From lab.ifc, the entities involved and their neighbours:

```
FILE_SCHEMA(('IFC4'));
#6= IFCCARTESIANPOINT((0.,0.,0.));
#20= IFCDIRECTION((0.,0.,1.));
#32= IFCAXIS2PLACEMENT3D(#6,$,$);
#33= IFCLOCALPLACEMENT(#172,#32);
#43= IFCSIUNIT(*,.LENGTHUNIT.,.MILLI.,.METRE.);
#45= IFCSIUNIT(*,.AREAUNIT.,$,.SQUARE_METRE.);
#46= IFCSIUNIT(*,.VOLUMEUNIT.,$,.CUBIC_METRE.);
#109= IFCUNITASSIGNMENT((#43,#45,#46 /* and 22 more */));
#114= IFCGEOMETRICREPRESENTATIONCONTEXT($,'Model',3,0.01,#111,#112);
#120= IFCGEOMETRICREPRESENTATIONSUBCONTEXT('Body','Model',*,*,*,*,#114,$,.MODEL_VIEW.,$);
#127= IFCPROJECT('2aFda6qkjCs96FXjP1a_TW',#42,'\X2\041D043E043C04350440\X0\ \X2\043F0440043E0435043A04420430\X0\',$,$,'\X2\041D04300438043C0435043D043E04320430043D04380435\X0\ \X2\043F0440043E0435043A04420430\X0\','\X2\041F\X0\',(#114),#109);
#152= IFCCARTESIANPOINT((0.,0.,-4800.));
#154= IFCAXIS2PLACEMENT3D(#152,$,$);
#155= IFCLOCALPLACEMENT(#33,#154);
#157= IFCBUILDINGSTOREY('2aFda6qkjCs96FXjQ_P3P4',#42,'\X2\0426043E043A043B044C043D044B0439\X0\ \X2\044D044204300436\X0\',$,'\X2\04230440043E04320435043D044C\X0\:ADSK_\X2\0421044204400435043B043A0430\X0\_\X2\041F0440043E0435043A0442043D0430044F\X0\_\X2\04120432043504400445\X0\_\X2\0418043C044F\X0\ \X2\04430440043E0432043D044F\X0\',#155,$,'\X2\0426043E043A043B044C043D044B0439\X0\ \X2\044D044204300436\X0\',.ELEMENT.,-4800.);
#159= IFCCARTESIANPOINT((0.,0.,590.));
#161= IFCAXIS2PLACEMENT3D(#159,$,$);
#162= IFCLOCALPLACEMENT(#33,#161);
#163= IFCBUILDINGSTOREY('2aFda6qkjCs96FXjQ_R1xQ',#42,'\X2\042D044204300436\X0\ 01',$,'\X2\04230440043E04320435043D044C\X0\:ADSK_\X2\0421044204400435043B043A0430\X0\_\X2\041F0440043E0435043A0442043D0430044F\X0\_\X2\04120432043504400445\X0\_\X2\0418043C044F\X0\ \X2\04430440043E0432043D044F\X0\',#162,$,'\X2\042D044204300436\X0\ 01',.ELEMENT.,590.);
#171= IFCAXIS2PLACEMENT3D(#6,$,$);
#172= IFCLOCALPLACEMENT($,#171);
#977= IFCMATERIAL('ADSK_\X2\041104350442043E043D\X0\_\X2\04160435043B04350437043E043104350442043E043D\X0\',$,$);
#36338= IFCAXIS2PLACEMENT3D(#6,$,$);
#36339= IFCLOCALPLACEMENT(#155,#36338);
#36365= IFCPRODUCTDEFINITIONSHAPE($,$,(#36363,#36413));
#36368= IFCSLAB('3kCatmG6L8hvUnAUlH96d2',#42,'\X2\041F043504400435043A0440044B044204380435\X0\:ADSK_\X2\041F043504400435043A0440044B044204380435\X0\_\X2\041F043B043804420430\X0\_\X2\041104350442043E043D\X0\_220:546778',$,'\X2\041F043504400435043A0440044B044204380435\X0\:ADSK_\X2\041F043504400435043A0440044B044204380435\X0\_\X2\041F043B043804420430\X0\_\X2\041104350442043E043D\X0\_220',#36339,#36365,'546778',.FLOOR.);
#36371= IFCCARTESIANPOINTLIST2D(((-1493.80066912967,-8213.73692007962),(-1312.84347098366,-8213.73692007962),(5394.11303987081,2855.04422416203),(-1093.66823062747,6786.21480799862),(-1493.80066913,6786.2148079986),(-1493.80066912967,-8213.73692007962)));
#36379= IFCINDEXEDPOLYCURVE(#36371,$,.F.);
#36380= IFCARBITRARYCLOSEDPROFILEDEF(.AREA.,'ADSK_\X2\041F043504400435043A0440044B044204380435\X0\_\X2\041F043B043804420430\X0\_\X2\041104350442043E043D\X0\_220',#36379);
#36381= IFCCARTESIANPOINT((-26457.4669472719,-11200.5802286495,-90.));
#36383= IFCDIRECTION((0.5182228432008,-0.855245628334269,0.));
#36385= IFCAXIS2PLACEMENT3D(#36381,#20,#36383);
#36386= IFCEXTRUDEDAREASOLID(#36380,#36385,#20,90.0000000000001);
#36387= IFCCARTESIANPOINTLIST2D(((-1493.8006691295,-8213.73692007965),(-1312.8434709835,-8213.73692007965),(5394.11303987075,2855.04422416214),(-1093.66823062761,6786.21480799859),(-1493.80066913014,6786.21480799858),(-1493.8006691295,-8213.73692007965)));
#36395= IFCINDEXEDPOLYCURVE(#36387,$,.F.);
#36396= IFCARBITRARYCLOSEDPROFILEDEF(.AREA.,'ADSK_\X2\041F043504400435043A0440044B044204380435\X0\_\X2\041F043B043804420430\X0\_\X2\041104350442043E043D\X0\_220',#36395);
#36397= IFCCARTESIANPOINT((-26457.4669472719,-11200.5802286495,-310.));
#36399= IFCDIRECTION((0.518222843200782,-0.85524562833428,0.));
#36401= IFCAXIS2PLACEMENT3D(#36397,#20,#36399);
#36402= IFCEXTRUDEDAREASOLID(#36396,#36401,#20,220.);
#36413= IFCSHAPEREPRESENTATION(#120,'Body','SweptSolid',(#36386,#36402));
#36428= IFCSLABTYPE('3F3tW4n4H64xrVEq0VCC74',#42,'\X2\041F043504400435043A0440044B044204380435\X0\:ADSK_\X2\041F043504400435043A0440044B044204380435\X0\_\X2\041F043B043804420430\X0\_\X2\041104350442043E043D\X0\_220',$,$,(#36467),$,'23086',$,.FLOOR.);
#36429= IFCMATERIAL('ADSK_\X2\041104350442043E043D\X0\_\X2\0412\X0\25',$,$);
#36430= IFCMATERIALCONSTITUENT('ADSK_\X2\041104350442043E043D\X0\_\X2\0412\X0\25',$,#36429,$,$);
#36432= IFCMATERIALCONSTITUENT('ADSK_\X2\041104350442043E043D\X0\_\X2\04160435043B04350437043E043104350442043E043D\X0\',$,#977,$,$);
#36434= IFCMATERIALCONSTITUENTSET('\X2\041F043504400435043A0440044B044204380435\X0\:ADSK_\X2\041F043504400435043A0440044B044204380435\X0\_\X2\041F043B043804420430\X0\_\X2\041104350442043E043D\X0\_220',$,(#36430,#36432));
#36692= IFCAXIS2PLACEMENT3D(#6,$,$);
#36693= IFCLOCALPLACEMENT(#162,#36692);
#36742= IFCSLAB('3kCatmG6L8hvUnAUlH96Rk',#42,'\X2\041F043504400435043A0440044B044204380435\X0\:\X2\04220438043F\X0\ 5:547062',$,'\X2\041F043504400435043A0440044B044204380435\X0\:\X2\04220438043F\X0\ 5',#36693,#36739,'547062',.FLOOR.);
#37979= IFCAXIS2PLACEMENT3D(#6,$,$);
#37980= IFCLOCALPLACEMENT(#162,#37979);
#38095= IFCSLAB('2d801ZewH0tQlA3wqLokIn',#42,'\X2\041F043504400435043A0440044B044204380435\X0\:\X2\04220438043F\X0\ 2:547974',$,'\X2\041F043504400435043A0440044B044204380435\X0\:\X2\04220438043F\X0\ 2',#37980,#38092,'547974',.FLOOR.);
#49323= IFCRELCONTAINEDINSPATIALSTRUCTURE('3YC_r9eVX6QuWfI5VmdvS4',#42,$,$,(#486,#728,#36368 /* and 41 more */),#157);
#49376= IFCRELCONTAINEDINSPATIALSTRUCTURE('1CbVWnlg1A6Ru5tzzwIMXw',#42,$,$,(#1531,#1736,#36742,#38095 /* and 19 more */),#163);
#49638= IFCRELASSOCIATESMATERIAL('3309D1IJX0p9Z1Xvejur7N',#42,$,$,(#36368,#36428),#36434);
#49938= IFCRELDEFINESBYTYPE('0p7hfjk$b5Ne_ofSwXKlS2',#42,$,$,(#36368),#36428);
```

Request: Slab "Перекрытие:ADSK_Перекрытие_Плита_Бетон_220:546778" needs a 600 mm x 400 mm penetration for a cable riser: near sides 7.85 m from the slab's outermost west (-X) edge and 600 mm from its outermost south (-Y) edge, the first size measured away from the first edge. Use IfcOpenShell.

```python
import numpy as np
import ifcopenshell
import ifcopenshell.api.feature
import ifcopenshell.api.geometry
import ifcopenshell.api.root
import ifcopenshell.geom
import ifcopenshell.util.placement
import ifcopenshell.util.representation
import ifcopenshell.util.shape
import ifcopenshell.util.unit

model = ifcopenshell.open("lab.ifc")
unit_scale = ifcopenshell.util.unit.calculate_unit_scale(model)
settings = ifcopenshell.geom.settings()


def volume(element):
    """Net volume in cubic metres, openings subtracted."""
    shape = ifcopenshell.geom.create_shape(settings, element)
    return ifcopenshell.util.shape.get_volume(shape.geometry)


slab = model.by_guid("3kCatmG6L8hvUnAUlH96d2")
before = volume(slab)

# Extent in the slab's own axes, in metres. The edges named are its -X and -Y sides.
slab_shape = ifcopenshell.geom.create_shape(settings, slab)
vertices = ifcopenshell.util.shape.get_vertices(slab_shape.geometry)
x_min, y_min, bottom = vertices.min(axis=0)
top = vertices[:, 2].max()

opening = ifcopenshell.api.root.create_entity(model, ifc_class="IfcOpeningElement", name="Cable riser opening", predefined_type="OPENING")
context = ifcopenshell.util.representation.get_context(model, "Model", "Body", "MODEL_VIEW")
width, depth = 0.6, 0.4
outline = [(0.0, 0.0), (width, 0.0), (width, depth), (0.0, depth), (0.0, 0.0)]
# Overshoot both faces by 50 mm so the cut is clean.
shape = ifcopenshell.api.geometry.add_slab_representation(
    model, context=context, depth=top - bottom + 0.1, polyline=outline
)
ifcopenshell.api.geometry.assign_representation(model, product=opening, representation=shape)

matrix = ifcopenshell.util.placement.get_local_placement(slab.ObjectPlacement)
matrix[:, 3] = matrix @ np.append(np.array([x_min + 7.85, y_min + 0.6, bottom - 0.05]) / unit_scale, 1.0)
ifcopenshell.api.geometry.edit_object_placement(model, product=opening, matrix=matrix, is_si=False)
ifcopenshell.api.feature.add_feature(model, feature=opening, element=slab)

after = volume(slab)

print(f"slab volume {before:.3f} -> {after:.3f} m3")

model.write("lab_rev.ifc")
```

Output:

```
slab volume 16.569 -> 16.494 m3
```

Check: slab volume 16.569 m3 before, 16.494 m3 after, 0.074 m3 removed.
